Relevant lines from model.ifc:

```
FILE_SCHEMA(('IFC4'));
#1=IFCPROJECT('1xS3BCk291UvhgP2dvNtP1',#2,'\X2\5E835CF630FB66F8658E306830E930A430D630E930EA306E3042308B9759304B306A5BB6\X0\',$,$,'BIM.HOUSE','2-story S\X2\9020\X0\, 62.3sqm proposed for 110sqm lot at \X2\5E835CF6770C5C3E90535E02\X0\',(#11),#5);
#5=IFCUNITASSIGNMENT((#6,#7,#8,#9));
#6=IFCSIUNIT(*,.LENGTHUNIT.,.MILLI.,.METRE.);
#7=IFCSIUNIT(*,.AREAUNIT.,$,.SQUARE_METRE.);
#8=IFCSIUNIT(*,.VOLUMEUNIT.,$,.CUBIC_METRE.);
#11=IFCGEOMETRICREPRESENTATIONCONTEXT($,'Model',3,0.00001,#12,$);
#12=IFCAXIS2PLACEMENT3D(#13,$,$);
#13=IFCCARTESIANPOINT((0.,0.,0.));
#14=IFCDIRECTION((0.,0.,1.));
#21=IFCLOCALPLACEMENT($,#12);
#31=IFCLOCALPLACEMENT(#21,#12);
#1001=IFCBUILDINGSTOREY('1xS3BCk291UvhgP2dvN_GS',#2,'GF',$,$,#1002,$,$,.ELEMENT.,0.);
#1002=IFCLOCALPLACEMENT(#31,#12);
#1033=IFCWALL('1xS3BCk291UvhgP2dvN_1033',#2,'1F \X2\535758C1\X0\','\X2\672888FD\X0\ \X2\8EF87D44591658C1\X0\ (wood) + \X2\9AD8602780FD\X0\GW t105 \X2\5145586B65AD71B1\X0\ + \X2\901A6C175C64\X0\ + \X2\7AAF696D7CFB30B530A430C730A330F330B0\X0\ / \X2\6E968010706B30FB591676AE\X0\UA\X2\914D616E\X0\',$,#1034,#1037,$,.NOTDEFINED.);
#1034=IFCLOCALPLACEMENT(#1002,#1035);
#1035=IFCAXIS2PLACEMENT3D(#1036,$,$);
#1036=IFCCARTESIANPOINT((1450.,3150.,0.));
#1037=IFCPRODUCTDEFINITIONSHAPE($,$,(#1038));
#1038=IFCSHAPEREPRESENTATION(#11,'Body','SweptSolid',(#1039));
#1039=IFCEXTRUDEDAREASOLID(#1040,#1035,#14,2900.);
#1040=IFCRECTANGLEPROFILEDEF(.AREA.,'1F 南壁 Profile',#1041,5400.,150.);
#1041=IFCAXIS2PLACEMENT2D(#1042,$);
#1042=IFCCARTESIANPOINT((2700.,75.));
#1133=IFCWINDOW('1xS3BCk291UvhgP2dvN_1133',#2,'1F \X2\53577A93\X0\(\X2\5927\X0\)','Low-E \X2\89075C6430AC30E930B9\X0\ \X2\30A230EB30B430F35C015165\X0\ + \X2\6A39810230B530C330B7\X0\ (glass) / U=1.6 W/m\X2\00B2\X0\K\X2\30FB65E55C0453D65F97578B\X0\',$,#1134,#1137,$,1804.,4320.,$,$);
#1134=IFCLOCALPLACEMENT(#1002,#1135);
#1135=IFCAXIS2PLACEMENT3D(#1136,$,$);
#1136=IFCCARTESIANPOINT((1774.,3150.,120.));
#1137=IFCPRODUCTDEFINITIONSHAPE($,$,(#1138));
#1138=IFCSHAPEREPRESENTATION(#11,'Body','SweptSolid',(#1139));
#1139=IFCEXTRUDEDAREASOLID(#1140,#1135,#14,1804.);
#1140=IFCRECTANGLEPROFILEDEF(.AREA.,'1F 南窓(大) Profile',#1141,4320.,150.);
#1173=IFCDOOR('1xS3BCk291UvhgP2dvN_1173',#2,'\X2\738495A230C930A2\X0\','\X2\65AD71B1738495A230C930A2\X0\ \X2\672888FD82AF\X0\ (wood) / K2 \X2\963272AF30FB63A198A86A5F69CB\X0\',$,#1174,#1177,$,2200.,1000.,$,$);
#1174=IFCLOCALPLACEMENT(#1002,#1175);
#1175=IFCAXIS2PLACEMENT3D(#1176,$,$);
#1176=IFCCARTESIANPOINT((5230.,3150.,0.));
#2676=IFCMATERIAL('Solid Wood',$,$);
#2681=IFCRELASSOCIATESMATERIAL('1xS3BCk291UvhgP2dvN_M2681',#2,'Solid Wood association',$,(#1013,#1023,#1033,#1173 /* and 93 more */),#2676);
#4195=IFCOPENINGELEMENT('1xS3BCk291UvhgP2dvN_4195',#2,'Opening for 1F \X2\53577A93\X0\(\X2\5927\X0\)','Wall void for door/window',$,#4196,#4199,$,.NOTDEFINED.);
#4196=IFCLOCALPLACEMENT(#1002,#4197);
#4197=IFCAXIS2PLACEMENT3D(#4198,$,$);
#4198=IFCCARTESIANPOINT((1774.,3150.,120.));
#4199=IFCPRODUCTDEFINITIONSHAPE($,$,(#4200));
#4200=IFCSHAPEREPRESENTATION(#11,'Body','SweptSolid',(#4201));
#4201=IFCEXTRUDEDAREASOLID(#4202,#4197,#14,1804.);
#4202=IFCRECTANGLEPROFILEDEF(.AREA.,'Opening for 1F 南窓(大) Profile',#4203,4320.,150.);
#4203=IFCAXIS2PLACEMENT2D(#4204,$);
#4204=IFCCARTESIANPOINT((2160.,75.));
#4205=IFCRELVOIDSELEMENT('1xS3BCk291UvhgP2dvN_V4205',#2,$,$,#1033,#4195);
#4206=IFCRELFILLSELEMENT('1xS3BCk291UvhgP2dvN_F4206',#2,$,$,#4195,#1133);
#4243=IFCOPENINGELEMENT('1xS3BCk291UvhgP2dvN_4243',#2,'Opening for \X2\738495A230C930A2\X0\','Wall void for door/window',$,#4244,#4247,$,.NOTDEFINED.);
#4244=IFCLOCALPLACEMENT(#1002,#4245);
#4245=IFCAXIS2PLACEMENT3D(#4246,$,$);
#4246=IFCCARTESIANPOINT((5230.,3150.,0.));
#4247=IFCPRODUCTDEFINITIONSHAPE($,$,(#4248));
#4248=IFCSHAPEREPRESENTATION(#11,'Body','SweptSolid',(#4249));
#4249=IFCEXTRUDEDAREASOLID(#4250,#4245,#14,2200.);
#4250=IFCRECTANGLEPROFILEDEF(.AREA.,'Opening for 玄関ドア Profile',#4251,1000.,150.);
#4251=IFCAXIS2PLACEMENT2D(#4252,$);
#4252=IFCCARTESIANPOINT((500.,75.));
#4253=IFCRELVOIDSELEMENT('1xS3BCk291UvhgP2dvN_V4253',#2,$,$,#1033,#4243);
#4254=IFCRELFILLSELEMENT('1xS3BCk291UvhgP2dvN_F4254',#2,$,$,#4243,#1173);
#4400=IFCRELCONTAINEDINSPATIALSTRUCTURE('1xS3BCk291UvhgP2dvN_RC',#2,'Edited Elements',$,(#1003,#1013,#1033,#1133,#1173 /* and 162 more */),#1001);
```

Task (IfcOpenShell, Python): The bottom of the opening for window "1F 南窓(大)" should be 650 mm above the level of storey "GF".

```python
import numpy as np
import ifcopenshell
import ifcopenshell.api.geometry
import ifcopenshell.geom
import ifcopenshell.util.element
import ifcopenshell.util.placement
import ifcopenshell.util.shape
import ifcopenshell.util.unit

model = ifcopenshell.open("model.ifc")
unit_scale = ifcopenshell.util.unit.calculate_unit_scale(model)

window = model.by_guid("1xS3BCk291UvhgP2dvN_1133")
opening = window.FillsVoids[0].RelatingOpeningElement
storey = ifcopenshell.util.element.get_container(window, ifc_class="IfcBuildingStorey")
level = ifcopenshell.util.placement.get_local_placement(storey.ObjectPlacement)[2, 3]

# The opening's origin need not be at the sill, so measure its lowest point.
shape = ifcopenshell.geom.create_shape(ifcopenshell.geom.settings(), opening)
bottom = ifcopenshell.util.shape.get_shape_bottom_elevation(shape, shape.geometry) / unit_scale
dz = level + 0.65 / unit_scale - bottom

shift = np.array([0.0, 0.0, dz])
# The window is not placed relative to its opening, so move both.
for product in (opening, window):
    matrix = ifcopenshell.util.placement.get_local_placement(product.ObjectPlacement)
    matrix[:3, 3] += shift
    ifcopenshell.api.geometry.edit_object_placement(model, product=product, matrix=matrix, is_si=False)

print(f"moved by {dz * unit_scale:+.3f} m")

model.write("model_v2.ifc")
```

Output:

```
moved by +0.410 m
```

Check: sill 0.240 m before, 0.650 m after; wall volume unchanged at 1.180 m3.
